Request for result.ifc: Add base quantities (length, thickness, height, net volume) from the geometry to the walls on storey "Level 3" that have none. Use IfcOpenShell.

First a look at what the model holds.

```python
import ifcopenshell
import ifcopenshell.util.element
import ifcopenshell.util.unit

model = ifcopenshell.open("result.ifc")
print(model.schema)
for unit_type in ("LENGTHUNIT", "AREAUNIT", "VOLUMEUNIT"):
    print(unit_type, ifcopenshell.util.unit.calculate_unit_scale(model, unit_type))
storey = next(s for s in model.by_type("IfcBuildingStorey") if s.Name == "Level 3")
walls = [e for e in ifcopenshell.util.element.get_decomposition(storey) if e.is_a("IfcWall")]
for e in sorted(walls, key=lambda e: e.id()):
    print(e.id(), e.is_a(), e.Name, list(ifcopenshell.util.element.get_psets(e, qtos_only=True)), sep=" | ")
```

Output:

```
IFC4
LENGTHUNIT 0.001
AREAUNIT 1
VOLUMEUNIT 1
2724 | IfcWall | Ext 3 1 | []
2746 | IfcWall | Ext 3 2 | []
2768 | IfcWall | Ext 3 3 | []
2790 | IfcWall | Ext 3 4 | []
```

```python
import ifcopenshell
import ifcopenshell.api.pset
import ifcopenshell.geom
import ifcopenshell.util.element
import ifcopenshell.util.shape
import ifcopenshell.util.unit

model = ifcopenshell.open("result.ifc")
unit_scale = ifcopenshell.util.unit.calculate_unit_scale(model)
volume_scale = ifcopenshell.util.unit.calculate_unit_scale(model, "VOLUMEUNIT")
settings = ifcopenshell.geom.settings()

storey = next(s for s in model.by_type("IfcBuildingStorey") if s.Name == "Level 3")
walls = [e for e in ifcopenshell.util.element.get_decomposition(storey) if e.is_a("IfcWall")]

for e in sorted(walls, key=lambda e: e.id()):
    if ifcopenshell.util.element.get_psets(e, qtos_only=True, should_inherit=False):
        continue
    # Geometry comes back in metres, in the element's own axes.
    shape = ifcopenshell.geom.create_shape(settings, e)
    values = {
        "Length": ifcopenshell.util.shape.get_x(shape.geometry) / unit_scale,
        "Width": ifcopenshell.util.shape.get_y(shape.geometry) / unit_scale,
        "Height": ifcopenshell.util.shape.get_z(shape.geometry) / unit_scale,
        "NetVolume": ifcopenshell.util.shape.get_volume(shape.geometry) / volume_scale,
    }
    qto = ifcopenshell.api.pset.add_qto(model, product=e, name="Qto_WallBaseQuantities")
    ifcopenshell.api.pset.edit_qto(model, qto=qto, properties=values)
    print(e.id(), {k: round(v, 3) for k, v in values.items()})

model.write("result_rev.ifc")
```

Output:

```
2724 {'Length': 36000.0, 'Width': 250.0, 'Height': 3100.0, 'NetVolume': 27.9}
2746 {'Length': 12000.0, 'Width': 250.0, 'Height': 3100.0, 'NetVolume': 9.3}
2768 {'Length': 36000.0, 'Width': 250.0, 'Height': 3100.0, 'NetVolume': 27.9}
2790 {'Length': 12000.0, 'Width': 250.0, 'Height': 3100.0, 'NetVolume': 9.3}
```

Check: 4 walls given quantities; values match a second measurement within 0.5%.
